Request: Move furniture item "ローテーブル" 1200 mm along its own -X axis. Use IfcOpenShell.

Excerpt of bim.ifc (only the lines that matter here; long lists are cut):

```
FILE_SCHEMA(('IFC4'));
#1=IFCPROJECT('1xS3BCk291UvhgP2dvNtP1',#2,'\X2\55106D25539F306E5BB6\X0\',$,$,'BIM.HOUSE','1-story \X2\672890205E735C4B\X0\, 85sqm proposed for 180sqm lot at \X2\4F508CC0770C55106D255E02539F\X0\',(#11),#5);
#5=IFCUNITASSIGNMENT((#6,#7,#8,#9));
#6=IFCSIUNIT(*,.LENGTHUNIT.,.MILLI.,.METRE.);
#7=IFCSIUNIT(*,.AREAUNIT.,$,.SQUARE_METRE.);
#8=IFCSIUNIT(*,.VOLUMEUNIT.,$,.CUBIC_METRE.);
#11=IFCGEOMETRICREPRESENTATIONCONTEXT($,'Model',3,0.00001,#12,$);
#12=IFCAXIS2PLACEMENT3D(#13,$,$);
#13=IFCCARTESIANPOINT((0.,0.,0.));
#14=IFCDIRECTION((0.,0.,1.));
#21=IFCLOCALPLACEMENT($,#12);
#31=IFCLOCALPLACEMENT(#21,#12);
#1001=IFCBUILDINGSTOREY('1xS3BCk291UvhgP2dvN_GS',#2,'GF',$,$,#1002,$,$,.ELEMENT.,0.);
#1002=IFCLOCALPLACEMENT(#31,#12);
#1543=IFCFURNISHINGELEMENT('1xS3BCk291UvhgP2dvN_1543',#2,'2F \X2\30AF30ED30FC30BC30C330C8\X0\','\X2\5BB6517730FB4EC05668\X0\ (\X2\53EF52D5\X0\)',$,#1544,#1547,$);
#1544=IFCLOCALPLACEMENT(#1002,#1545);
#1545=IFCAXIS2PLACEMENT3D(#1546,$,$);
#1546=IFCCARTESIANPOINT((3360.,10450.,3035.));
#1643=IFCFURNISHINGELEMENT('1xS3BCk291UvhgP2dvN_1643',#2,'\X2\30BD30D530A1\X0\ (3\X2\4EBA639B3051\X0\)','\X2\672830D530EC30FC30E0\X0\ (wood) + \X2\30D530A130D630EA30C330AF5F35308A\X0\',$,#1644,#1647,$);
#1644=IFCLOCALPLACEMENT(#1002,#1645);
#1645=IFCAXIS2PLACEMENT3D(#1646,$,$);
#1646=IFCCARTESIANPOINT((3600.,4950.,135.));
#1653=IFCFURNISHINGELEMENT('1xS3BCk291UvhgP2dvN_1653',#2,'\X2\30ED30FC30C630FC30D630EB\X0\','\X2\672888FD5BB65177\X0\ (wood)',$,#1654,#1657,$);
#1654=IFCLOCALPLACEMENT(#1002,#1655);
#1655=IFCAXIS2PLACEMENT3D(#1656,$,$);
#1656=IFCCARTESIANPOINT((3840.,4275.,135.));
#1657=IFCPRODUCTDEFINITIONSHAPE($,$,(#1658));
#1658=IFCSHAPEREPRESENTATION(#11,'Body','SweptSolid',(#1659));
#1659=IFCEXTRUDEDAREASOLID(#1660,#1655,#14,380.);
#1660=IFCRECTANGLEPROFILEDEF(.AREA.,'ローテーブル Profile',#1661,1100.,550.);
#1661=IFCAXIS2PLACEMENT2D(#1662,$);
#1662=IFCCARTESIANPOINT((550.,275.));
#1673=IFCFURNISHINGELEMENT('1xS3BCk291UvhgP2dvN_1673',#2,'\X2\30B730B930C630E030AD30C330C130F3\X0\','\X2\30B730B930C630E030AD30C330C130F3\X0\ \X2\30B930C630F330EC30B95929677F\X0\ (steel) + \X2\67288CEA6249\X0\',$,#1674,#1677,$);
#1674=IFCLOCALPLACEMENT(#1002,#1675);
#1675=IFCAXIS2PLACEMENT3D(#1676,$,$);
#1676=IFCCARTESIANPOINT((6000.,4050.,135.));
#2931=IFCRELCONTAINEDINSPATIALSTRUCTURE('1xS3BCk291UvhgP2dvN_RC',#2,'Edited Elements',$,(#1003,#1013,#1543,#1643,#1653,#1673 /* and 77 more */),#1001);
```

```python
import ifcopenshell
import ifcopenshell.api.geometry
import ifcopenshell.util.placement

model = ifcopenshell.open("bim.ifc")

item = model.by_guid("1xS3BCk291UvhgP2dvN_1653")
matrix = ifcopenshell.util.placement.get_local_placement(item.ObjectPlacement)
matrix[:3, 3] -= matrix[:3, 0] * 1200.0
ifcopenshell.api.geometry.edit_object_placement(model, product=item, matrix=matrix, is_si=False)

print(ifcopenshell.util.placement.get_local_placement(item.ObjectPlacement).round(3) + 0.0)

model.write("bim-out.ifc")
```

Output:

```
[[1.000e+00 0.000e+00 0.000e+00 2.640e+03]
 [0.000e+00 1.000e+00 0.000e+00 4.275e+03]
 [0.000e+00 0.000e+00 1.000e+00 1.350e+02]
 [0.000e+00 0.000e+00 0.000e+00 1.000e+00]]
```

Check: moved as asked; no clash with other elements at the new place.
